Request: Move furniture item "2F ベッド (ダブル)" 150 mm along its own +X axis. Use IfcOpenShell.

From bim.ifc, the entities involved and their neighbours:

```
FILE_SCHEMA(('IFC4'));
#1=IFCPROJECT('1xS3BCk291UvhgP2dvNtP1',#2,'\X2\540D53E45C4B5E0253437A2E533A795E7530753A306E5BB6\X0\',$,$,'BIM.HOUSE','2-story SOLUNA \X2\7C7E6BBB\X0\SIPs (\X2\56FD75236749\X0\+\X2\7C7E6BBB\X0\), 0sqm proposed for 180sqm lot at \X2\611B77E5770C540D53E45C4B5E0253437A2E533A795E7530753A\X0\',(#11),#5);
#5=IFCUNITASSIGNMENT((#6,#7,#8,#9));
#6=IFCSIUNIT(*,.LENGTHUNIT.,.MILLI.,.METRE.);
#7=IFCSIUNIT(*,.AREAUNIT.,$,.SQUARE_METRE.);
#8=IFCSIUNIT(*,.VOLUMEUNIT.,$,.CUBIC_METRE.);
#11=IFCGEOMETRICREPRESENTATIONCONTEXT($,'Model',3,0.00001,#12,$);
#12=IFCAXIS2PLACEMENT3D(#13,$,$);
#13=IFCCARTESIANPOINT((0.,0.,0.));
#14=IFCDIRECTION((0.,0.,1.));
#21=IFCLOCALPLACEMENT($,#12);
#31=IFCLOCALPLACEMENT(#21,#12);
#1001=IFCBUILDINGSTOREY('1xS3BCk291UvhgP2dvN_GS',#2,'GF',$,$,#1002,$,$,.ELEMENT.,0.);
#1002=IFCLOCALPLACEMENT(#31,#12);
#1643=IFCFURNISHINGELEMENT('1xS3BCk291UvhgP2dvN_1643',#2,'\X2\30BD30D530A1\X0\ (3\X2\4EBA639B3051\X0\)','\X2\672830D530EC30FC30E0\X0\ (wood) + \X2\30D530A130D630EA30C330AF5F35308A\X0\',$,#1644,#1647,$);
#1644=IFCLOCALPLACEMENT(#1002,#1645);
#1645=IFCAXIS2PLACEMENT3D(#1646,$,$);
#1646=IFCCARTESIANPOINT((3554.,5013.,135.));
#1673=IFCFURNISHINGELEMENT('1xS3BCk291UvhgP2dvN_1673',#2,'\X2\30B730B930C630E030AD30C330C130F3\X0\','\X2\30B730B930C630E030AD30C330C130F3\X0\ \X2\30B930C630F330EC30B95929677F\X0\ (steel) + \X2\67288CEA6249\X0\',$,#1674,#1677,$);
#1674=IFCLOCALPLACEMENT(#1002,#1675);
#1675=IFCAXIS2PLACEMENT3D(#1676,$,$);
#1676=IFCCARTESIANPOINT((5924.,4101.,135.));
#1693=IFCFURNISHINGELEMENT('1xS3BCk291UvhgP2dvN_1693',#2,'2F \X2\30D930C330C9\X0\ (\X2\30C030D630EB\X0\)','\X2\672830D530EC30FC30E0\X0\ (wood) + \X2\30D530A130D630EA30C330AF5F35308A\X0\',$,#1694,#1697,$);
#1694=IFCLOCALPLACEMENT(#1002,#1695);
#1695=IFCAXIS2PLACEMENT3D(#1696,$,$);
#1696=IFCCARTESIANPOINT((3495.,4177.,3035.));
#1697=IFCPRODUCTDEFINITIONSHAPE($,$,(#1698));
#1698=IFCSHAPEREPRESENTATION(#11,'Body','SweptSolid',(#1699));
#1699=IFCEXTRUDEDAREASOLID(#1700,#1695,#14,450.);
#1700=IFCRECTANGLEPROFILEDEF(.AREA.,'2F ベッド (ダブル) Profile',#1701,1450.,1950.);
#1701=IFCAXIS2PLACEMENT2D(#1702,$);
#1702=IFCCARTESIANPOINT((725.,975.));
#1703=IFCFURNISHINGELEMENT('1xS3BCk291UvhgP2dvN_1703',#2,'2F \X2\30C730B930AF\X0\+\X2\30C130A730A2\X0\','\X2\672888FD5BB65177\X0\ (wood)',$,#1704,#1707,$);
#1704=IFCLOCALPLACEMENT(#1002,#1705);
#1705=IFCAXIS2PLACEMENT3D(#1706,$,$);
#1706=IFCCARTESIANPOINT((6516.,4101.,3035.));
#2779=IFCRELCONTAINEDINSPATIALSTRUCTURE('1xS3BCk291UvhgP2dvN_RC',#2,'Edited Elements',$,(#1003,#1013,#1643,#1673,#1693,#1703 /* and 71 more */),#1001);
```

```python
import ifcopenshell
import ifcopenshell.api.geometry
import ifcopenshell.util.placement
import ifcopenshell.util.unit

model = ifcopenshell.open("bim.ifc")
unit_scale = ifcopenshell.util.unit.calculate_unit_scale(model)

item = model.by_guid("1xS3BCk291UvhgP2dvN_1693")
matrix = ifcopenshell.util.placement.get_local_placement(item.ObjectPlacement)
matrix[:3, 3] += matrix[:3, 0] * 0.15 / unit_scale
ifcopenshell.api.geometry.edit_object_placement(model, product=item, matrix=matrix, is_si=False)

print(ifcopenshell.util.placement.get_local_placement(item.ObjectPlacement).round(3) + 0.0)

model.write("bim_rev.ifc")
```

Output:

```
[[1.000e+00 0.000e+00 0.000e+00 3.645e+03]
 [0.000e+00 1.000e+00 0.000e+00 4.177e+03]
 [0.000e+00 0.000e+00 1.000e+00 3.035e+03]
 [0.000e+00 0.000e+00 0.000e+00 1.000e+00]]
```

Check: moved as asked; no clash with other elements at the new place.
